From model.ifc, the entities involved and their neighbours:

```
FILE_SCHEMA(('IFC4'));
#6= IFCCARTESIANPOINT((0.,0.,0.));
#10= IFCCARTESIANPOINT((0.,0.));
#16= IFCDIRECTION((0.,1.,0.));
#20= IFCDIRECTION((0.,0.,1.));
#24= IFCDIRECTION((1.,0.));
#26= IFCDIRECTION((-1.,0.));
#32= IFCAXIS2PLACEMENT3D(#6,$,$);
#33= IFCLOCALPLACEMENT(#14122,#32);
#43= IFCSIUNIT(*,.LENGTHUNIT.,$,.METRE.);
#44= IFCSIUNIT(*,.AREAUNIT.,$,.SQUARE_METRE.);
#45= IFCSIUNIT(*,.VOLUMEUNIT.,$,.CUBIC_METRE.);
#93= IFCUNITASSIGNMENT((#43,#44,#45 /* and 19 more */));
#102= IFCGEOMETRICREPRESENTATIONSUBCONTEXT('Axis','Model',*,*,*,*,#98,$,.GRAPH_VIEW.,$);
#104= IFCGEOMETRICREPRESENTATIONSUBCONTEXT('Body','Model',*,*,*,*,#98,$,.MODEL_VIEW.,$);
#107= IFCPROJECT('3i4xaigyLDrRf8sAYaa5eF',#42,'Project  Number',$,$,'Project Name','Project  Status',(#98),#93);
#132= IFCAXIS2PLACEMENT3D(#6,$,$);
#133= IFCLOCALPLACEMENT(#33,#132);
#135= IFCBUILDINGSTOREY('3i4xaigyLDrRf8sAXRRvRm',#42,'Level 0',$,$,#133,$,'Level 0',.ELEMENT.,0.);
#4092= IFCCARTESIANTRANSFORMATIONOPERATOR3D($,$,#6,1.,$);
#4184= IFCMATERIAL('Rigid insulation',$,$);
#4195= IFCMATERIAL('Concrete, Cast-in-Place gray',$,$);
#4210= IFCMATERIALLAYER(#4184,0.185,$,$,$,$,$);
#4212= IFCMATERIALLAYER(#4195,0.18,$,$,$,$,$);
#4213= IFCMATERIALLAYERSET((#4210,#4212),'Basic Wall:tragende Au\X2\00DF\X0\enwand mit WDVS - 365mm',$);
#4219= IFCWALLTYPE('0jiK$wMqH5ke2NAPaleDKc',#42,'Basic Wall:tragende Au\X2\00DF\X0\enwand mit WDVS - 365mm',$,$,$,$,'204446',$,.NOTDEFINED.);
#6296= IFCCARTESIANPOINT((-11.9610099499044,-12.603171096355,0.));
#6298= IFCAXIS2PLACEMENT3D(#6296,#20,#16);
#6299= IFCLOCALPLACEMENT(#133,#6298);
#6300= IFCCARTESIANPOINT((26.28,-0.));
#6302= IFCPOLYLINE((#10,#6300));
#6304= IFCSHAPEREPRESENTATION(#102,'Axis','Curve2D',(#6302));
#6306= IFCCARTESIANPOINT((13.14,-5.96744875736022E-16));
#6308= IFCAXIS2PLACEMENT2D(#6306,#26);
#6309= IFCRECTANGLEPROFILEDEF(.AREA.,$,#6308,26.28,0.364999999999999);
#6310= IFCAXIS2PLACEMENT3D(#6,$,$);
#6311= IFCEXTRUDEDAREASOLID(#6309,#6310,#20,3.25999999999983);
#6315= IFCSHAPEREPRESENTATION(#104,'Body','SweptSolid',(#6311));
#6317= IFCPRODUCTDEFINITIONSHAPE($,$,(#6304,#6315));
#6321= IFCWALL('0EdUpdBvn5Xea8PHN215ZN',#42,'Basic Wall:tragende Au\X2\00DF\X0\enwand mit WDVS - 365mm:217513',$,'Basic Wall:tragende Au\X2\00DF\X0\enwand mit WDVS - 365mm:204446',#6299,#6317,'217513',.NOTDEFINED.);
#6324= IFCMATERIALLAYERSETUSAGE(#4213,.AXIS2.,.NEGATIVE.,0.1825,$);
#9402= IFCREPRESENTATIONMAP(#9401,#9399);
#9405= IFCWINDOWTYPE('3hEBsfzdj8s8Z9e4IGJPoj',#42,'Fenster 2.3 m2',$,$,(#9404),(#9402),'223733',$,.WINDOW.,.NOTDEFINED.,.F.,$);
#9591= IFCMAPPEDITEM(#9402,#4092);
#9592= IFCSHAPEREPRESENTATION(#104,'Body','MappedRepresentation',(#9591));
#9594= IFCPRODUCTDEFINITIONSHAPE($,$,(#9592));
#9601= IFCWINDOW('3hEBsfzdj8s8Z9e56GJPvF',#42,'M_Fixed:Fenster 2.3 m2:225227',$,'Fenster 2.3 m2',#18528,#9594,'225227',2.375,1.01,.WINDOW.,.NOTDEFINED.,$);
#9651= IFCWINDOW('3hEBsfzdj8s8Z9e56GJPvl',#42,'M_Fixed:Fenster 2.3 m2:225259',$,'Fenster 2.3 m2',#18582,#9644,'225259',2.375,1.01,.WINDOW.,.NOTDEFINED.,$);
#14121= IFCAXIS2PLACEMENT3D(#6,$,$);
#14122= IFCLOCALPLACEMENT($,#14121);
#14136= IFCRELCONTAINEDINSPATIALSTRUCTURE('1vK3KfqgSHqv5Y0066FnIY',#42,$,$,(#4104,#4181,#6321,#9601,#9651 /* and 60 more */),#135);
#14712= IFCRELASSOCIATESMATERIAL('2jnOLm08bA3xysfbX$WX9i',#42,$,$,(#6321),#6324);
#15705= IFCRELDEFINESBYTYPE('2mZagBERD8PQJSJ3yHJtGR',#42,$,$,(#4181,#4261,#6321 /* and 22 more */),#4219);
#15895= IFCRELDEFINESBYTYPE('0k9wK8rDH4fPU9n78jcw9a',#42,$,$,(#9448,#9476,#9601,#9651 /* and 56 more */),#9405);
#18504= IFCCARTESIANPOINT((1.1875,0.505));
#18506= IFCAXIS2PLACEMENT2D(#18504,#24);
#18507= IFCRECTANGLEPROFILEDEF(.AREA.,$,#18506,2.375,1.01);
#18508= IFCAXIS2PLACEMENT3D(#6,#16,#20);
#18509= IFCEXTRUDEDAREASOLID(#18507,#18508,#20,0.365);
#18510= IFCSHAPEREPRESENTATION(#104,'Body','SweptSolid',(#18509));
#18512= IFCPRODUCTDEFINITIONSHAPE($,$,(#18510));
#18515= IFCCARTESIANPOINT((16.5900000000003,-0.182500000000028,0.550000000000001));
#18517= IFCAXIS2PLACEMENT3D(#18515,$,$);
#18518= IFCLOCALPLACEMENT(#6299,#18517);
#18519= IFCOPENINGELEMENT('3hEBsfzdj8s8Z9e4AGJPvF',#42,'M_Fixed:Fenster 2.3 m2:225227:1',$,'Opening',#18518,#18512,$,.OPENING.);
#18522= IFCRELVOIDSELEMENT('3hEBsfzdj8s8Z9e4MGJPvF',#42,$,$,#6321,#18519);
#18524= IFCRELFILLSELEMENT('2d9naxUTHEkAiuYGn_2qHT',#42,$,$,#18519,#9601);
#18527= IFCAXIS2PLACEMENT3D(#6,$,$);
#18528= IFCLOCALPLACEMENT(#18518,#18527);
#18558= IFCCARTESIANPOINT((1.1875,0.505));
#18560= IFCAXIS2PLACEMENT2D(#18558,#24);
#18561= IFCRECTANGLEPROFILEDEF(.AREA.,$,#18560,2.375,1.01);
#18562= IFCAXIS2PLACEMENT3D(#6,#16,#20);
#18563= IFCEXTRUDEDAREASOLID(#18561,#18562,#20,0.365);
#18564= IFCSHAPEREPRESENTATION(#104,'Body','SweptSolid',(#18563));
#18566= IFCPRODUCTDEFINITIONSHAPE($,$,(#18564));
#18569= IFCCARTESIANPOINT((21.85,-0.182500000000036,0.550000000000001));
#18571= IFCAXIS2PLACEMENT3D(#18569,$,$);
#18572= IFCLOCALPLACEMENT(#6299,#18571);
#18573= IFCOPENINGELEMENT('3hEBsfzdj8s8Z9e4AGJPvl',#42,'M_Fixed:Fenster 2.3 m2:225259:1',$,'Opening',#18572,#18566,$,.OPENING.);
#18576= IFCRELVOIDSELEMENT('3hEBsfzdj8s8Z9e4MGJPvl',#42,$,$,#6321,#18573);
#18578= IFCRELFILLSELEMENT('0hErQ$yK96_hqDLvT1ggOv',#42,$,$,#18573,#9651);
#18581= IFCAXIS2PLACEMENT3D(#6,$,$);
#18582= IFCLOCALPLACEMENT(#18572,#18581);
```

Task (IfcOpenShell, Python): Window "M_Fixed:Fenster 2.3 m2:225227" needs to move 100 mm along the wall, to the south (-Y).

```python
import ifcopenshell
import ifcopenshell.api.geometry
import ifcopenshell.util.placement

model = ifcopenshell.open("model.ifc")

window = model.by_guid("3hEBsfzdj8s8Z9e56GJPvF")
opening = window.FillsVoids[0].RelatingOpeningElement
wall = opening.VoidsElements[0].RelatingBuildingElement

wall_matrix = ifcopenshell.util.placement.get_local_placement(wall.ObjectPlacement)
shift = wall_matrix[:3, 0] * -0.1
before = ifcopenshell.util.placement.get_local_placement(window.ObjectPlacement)[:3, 3].copy()

# The window is placed relative to its opening, so it follows when the opening moves.
matrix = ifcopenshell.util.placement.get_local_placement(opening.ObjectPlacement)
matrix[:3, 3] += shift
ifcopenshell.api.geometry.edit_object_placement(
    model, product=opening, matrix=matrix, is_si=False, should_transform_children=True
)

after = ifcopenshell.util.placement.get_local_placement(window.ObjectPlacement)[:3, 3]
print("window moved by", (after - before).round(3) + 0.0)

model.write("model_v2.ifc")
```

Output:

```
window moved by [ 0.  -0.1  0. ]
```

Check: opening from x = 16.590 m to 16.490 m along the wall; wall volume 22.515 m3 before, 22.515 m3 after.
